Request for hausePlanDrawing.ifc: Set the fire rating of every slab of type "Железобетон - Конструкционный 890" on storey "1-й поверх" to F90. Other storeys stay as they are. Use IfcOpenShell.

First a look at what the model holds.

```python
import ifcopenshell
import ifcopenshell.util.element

model = ifcopenshell.open("hausePlanDrawing.ifc")
print(model.schema)
storey = next(s for s in model.by_type("IfcBuildingStorey") if s.Name == "1-й поверх")
slabs = [e for e in ifcopenshell.util.element.get_decomposition(storey) if e.is_a("IfcSlab")]
seen = {}
for e in slabs:
    element_type = ifcopenshell.util.element.get_type(e)
    key = (element_type.Name if element_type != e and element_type else None, ifcopenshell.util.element.get_pset(e, "Pset_SlabCommon", "FireRating"))
    seen[key] = seen.get(key, 0) + 1
for (name, value), count in sorted(seen.items(), key=str):
    print(count, "x", name, "|", value)
```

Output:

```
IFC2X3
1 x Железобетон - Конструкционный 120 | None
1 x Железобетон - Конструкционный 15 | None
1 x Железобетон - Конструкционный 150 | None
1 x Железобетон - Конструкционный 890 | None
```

```python
import ifcopenshell
import ifcopenshell.api.pset
import ifcopenshell.util.element

model = ifcopenshell.open("hausePlanDrawing.ifc")

storey = next(s for s in model.by_type("IfcBuildingStorey") if s.Name == "1-й поверх")
slabs = [e for e in ifcopenshell.util.element.get_decomposition(storey) if e.is_a("IfcSlab")]

count = 0
for e in slabs:
    element_type = ifcopenshell.util.element.get_type(e)
    if element_type in (None, e) or element_type.Name != "Железобетон - Конструкционный 890":
        continue
    # add_pset returns the element's existing set when there is one.
    pset = ifcopenshell.api.pset.add_pset(model, product=e, name="Pset_SlabCommon")
    ifcopenshell.api.pset.edit_pset(model, pset=pset, properties={"FireRating": "F90"})
    count += 1

print(count, "slabs updated")

model.write("hausePlanDrawing_updated.ifc")
```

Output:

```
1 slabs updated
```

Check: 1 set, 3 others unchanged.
